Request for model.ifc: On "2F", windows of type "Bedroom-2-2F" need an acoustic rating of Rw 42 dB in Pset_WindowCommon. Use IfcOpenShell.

First a look at what the model holds.

```python
import ifcopenshell
import ifcopenshell.util.element

model = ifcopenshell.open("model.ifc")
print(model.schema)
storey = next(s for s in model.by_type("IfcBuildingStorey") if s.Name == "2F")
windows = [e for e in ifcopenshell.util.element.get_decomposition(storey) if e.is_a("IfcWindow")]
seen = {}
for e in windows:
    element_type = ifcopenshell.util.element.get_type(e)
    key = (element_type.Name if element_type != e and element_type else None, ifcopenshell.util.element.get_pset(e, "Pset_WindowCommon", "AcousticRating"))
    seen[key] = seen.get(key, 0) + 1
for (name, value), count in sorted(seen.items(), key=str):
    print(count, "x", name, "|", value)
```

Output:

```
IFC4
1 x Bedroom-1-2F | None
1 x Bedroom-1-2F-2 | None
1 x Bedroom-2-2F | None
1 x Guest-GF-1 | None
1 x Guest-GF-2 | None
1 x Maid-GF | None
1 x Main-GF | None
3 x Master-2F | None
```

```python
import ifcopenshell
import ifcopenshell.api.pset
import ifcopenshell.util.element

model = ifcopenshell.open("model.ifc")

storey = next(s for s in model.by_type("IfcBuildingStorey") if s.Name == "2F")
windows = [e for e in ifcopenshell.util.element.get_decomposition(storey) if e.is_a("IfcWindow")]

count = 0
for e in windows:
    element_type = ifcopenshell.util.element.get_type(e)
    if element_type in (None, e) or element_type.Name != "Bedroom-2-2F":
        continue
    # add_pset returns the element's existing set when there is one.
    pset = ifcopenshell.api.pset.add_pset(model, product=e, name="Pset_WindowCommon")
    ifcopenshell.api.pset.edit_pset(model, pset=pset, properties={"AcousticRating": "Rw 42 dB"})
    count += 1

print(count, "windows updated")

model.write("model_rev.ifc")
```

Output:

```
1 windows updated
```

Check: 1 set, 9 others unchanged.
